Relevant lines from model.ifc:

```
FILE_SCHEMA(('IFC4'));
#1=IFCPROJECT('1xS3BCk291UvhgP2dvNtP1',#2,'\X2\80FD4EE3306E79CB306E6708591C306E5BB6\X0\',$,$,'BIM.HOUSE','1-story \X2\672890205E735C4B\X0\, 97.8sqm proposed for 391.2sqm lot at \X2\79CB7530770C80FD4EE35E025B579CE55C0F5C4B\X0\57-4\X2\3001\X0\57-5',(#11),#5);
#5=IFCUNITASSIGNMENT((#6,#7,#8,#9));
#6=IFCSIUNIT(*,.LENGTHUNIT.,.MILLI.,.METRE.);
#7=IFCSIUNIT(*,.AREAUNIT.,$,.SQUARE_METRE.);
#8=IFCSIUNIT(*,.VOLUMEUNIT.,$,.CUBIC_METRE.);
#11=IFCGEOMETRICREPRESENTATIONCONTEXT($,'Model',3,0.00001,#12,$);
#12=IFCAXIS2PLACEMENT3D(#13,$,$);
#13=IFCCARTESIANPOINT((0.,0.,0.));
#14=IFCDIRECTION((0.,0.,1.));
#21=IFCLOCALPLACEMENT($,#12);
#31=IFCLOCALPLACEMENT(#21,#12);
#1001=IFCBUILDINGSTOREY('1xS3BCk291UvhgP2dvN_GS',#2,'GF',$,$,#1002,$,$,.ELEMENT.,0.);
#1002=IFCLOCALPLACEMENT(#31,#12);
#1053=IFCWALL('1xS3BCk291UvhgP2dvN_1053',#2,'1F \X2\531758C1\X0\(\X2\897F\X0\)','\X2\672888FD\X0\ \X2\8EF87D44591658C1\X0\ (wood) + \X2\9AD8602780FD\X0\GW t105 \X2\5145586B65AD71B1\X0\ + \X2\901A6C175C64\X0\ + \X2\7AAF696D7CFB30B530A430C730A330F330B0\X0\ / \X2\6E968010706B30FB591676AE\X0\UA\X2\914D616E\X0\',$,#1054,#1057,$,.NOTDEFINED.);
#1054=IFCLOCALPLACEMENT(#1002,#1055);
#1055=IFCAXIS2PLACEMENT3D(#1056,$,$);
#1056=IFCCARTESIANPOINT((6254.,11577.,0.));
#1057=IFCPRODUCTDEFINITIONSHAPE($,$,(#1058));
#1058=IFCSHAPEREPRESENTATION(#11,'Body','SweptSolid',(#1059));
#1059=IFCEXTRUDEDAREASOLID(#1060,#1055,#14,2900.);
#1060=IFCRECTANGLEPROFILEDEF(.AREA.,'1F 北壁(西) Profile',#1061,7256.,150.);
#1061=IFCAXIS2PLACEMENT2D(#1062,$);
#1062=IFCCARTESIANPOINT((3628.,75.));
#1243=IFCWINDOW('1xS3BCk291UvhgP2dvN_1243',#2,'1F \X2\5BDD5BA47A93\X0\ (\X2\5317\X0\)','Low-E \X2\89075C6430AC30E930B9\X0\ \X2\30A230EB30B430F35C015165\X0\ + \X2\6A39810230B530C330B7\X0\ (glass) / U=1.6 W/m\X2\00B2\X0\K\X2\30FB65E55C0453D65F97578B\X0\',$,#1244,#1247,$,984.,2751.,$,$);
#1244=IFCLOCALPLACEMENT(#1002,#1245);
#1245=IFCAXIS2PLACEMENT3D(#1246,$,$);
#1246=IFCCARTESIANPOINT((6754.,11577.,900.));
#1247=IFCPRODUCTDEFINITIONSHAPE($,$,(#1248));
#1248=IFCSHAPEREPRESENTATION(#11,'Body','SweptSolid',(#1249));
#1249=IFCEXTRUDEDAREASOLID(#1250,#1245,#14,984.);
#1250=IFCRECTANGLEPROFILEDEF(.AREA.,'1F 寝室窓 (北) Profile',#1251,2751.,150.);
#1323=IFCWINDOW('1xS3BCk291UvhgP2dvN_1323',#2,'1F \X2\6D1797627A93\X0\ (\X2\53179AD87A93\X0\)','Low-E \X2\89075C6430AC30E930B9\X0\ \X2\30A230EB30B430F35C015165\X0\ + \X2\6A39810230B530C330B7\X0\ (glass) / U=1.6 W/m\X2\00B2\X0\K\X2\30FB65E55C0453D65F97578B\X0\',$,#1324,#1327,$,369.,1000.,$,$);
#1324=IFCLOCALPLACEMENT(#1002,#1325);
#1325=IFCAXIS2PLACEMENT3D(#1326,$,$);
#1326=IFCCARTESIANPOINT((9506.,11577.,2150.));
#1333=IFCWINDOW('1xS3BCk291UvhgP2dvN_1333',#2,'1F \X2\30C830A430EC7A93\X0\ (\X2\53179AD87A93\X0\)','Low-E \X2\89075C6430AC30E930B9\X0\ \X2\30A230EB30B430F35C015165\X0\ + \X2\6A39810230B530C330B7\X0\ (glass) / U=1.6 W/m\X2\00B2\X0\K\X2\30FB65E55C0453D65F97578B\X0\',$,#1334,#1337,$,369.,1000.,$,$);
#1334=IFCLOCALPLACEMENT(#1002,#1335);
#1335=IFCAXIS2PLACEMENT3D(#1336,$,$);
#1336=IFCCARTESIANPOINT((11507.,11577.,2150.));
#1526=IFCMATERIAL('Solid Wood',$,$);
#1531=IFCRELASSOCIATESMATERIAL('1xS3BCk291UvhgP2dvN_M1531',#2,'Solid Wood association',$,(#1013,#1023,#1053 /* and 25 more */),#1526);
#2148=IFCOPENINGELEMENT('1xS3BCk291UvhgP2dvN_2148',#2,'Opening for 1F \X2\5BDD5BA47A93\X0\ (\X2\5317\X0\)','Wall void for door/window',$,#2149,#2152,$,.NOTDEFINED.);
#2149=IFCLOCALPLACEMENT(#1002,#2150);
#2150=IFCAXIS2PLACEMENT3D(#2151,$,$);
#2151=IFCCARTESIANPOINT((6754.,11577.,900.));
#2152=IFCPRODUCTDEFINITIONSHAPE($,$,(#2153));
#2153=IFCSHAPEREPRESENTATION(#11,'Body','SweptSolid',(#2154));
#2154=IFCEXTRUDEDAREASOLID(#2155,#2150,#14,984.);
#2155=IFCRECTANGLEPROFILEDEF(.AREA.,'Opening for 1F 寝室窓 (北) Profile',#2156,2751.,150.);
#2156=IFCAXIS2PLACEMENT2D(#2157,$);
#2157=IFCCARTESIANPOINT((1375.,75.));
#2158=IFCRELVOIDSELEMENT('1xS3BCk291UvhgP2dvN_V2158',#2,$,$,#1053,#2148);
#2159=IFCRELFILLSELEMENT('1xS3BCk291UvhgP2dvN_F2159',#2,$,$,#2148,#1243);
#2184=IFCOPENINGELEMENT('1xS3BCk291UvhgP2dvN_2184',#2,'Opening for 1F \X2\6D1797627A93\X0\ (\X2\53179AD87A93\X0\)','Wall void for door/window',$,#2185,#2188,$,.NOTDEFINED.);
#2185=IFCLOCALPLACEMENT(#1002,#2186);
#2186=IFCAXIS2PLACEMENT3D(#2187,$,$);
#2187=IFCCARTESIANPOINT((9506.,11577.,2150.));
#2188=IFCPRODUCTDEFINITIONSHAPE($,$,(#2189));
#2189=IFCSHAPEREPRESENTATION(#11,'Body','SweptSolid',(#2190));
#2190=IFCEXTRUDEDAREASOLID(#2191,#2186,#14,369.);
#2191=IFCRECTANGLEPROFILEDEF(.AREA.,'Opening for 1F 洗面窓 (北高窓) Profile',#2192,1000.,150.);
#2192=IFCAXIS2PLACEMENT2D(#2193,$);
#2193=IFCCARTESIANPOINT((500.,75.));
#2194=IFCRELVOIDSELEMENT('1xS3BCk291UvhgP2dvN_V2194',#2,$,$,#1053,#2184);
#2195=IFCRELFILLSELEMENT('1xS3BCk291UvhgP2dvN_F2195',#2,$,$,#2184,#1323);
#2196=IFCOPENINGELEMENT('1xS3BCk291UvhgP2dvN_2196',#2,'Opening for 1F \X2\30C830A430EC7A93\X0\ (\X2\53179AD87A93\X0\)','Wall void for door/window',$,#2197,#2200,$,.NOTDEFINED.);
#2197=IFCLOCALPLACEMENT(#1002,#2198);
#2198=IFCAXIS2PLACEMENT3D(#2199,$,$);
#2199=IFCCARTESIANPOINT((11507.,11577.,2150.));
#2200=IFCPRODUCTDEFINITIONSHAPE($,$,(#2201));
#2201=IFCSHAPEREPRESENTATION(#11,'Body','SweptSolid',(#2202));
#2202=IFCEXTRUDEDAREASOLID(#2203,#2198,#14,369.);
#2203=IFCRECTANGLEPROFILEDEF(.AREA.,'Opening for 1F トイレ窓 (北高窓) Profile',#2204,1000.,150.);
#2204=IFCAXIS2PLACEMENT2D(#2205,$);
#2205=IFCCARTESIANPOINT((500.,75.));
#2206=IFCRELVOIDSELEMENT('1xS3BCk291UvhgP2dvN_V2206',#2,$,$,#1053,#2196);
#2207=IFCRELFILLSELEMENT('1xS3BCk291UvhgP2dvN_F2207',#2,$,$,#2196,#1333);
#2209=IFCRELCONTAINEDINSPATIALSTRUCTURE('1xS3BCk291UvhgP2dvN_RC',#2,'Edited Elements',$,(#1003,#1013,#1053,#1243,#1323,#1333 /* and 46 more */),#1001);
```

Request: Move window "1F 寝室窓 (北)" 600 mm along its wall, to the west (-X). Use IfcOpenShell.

```python
import ifcopenshell
import ifcopenshell.api.geometry
import ifcopenshell.util.placement
import ifcopenshell.util.unit

model = ifcopenshell.open("model.ifc")
unit_scale = ifcopenshell.util.unit.calculate_unit_scale(model)

window = model.by_guid("1xS3BCk291UvhgP2dvN_1243")
opening = window.FillsVoids[0].RelatingOpeningElement
wall = opening.VoidsElements[0].RelatingBuildingElement

wall_matrix = ifcopenshell.util.placement.get_local_placement(wall.ObjectPlacement)
shift = wall_matrix[:3, 0] * -0.6 / unit_scale
before = ifcopenshell.util.placement.get_local_placement(window.ObjectPlacement)[:3, 3].copy()

# The window is not placed relative to its opening, so move both.
for product in (opening, window):
    matrix = ifcopenshell.util.placement.get_local_placement(product.ObjectPlacement)
    matrix[:3, 3] += shift
    ifcopenshell.api.geometry.edit_object_placement(model, product=product, matrix=matrix, is_si=False)

after = ifcopenshell.util.placement.get_local_placement(window.ObjectPlacement)[:3, 3]
print("window moved by", (after - before).round(3) + 0.0)

model.write("model_updated.ifc")
```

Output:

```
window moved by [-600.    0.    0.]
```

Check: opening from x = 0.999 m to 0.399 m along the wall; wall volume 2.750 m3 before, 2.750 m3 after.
